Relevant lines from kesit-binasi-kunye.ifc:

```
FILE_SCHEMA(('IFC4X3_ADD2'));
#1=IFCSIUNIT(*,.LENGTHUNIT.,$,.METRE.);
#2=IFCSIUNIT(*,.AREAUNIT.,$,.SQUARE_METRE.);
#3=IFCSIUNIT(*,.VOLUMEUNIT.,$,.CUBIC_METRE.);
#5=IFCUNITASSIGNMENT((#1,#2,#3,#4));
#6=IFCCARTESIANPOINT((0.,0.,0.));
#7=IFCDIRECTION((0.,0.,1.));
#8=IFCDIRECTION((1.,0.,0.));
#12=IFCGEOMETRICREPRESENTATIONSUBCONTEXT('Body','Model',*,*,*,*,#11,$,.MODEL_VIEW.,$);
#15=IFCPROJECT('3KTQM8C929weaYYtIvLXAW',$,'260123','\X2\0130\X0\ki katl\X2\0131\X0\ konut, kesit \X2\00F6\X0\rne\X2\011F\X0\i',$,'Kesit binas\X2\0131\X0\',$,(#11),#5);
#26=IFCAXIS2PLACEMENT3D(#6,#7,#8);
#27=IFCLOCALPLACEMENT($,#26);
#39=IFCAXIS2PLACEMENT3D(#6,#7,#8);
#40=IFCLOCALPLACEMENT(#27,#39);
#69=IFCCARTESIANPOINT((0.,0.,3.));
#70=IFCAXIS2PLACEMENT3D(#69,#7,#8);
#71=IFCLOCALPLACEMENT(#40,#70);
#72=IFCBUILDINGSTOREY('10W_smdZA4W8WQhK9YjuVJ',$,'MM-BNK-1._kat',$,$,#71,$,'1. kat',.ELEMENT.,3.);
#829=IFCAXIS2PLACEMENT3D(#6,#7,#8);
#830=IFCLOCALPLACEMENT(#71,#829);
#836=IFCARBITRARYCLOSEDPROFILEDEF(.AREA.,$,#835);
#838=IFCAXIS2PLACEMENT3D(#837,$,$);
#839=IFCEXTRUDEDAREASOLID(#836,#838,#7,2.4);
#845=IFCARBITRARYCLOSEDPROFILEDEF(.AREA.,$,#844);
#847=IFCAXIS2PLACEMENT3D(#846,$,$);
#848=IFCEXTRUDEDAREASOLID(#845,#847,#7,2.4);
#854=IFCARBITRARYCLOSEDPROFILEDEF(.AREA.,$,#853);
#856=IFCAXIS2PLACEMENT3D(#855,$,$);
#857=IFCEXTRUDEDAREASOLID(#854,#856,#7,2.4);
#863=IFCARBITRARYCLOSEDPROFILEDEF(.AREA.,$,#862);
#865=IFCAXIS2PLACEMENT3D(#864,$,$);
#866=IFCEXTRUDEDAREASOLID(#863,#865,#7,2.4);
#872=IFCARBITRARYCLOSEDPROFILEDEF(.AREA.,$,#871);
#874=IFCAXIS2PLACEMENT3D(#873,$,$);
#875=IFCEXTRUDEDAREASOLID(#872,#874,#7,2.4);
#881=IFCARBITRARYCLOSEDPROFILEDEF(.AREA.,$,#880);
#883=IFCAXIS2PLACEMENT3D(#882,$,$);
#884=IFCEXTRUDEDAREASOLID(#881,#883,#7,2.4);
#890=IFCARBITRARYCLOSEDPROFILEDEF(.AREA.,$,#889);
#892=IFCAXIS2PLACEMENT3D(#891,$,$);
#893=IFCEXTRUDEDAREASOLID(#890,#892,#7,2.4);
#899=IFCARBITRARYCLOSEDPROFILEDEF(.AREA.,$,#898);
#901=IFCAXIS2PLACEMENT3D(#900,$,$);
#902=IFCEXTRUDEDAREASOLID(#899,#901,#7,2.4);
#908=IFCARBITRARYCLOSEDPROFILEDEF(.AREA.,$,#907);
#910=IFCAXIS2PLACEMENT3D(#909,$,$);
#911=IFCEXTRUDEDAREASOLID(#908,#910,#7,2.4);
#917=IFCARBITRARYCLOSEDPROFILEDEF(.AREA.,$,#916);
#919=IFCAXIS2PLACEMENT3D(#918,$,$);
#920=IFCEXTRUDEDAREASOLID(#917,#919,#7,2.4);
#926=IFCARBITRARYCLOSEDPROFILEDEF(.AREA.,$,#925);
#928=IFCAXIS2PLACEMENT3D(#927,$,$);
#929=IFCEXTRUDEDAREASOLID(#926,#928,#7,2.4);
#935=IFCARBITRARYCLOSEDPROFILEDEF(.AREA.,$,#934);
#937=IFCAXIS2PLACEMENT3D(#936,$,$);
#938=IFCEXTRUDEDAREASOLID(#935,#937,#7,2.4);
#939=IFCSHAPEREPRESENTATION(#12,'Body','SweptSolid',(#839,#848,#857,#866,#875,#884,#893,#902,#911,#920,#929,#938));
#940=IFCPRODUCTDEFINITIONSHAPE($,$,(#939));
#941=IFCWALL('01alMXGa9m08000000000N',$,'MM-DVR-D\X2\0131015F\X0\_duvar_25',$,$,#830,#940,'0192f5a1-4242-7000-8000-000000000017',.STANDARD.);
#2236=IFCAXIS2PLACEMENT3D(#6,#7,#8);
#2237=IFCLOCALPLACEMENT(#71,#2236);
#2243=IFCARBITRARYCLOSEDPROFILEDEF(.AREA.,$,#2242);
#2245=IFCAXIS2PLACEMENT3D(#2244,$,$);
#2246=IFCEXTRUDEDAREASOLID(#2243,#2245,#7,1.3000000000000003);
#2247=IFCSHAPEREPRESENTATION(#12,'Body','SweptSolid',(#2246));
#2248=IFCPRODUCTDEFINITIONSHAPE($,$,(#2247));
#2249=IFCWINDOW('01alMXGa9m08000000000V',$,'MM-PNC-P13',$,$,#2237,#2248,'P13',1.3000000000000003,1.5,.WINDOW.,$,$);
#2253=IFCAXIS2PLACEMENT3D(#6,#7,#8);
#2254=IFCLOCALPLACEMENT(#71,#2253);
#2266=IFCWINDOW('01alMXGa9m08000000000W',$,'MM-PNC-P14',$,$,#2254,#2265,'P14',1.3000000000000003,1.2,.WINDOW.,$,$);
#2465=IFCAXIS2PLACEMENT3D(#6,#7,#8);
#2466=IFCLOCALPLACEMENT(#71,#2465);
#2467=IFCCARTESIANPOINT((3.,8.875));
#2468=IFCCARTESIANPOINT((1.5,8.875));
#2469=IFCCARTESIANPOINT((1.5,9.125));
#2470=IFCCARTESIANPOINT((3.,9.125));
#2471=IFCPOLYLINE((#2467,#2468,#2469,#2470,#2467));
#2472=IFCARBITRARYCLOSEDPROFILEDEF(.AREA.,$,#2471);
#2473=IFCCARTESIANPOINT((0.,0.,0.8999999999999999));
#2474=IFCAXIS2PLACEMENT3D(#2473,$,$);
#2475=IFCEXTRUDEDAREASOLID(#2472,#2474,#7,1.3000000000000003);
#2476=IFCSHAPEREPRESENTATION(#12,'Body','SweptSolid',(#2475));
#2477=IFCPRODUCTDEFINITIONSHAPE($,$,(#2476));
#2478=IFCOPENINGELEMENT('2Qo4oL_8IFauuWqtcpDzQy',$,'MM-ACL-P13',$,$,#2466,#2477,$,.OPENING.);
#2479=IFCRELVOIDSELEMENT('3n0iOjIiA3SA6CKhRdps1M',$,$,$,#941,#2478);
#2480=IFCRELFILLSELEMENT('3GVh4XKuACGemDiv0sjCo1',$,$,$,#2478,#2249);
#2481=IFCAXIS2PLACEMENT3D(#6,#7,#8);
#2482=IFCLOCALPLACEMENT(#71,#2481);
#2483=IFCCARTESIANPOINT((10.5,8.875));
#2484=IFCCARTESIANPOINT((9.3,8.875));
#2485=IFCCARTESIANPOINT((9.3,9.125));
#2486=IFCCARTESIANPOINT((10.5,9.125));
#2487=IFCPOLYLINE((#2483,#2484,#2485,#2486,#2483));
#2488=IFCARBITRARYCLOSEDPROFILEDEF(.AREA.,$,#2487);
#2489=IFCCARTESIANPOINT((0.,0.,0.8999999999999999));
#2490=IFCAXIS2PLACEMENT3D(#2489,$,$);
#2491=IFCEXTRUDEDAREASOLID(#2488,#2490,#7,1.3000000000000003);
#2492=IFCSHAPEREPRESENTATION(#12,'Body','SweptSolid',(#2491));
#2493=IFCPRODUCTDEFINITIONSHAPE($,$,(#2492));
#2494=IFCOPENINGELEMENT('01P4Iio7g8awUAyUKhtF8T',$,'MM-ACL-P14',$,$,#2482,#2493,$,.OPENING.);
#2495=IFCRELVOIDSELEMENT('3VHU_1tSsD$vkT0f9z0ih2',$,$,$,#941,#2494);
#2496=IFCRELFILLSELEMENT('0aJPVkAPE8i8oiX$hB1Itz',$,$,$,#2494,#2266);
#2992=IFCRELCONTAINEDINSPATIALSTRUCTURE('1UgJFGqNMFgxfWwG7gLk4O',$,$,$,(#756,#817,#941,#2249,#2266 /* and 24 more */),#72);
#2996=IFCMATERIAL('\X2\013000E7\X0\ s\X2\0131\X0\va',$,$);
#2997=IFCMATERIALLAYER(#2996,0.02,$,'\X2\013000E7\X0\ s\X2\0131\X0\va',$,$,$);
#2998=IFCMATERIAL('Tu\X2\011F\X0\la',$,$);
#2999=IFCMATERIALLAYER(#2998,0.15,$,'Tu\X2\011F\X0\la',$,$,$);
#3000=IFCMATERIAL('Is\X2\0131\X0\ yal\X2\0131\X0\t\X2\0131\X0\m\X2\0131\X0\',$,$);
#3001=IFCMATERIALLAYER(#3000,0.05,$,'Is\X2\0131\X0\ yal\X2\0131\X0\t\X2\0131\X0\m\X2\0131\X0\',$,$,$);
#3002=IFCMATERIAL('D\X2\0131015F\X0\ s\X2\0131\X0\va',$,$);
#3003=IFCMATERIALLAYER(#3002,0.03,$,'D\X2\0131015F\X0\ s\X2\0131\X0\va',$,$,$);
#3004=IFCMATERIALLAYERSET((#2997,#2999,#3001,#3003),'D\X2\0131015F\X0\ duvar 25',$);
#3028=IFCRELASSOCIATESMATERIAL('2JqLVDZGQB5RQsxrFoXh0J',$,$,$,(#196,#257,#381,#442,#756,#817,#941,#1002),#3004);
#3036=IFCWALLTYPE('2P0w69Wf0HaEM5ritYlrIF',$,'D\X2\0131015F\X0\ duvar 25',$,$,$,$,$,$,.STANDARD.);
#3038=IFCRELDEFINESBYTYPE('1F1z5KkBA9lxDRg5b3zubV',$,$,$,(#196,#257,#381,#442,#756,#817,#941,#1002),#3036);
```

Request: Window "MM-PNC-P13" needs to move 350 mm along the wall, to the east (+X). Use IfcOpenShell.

```python
import ifcopenshell
import ifcopenshell.api.geometry
import ifcopenshell.util.placement

model = ifcopenshell.open("kesit-binasi-kunye.ifc")

window = model.by_guid("01alMXGa9m08000000000V")
opening = window.FillsVoids[0].RelatingOpeningElement
wall = opening.VoidsElements[0].RelatingBuildingElement

wall_matrix = ifcopenshell.util.placement.get_local_placement(wall.ObjectPlacement)
shift = wall_matrix[:3, 0] * 0.35
before = ifcopenshell.util.placement.get_local_placement(window.ObjectPlacement)[:3, 3].copy()

# The window is not placed relative to its opening, so move both.
for product in (opening, window):
    matrix = ifcopenshell.util.placement.get_local_placement(product.ObjectPlacement)
    matrix[:3, 3] += shift
    ifcopenshell.api.geometry.edit_object_placement(model, product=product, matrix=matrix, is_si=False)

after = ifcopenshell.util.placement.get_local_placement(window.ObjectPlacement)[:3, 3]
print("window moved by", (after - before).round(3) + 0.0)

model.write("kesit-binasi-kunye_rev.ifc")
```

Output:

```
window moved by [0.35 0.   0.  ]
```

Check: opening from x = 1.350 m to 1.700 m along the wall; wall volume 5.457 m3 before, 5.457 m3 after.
